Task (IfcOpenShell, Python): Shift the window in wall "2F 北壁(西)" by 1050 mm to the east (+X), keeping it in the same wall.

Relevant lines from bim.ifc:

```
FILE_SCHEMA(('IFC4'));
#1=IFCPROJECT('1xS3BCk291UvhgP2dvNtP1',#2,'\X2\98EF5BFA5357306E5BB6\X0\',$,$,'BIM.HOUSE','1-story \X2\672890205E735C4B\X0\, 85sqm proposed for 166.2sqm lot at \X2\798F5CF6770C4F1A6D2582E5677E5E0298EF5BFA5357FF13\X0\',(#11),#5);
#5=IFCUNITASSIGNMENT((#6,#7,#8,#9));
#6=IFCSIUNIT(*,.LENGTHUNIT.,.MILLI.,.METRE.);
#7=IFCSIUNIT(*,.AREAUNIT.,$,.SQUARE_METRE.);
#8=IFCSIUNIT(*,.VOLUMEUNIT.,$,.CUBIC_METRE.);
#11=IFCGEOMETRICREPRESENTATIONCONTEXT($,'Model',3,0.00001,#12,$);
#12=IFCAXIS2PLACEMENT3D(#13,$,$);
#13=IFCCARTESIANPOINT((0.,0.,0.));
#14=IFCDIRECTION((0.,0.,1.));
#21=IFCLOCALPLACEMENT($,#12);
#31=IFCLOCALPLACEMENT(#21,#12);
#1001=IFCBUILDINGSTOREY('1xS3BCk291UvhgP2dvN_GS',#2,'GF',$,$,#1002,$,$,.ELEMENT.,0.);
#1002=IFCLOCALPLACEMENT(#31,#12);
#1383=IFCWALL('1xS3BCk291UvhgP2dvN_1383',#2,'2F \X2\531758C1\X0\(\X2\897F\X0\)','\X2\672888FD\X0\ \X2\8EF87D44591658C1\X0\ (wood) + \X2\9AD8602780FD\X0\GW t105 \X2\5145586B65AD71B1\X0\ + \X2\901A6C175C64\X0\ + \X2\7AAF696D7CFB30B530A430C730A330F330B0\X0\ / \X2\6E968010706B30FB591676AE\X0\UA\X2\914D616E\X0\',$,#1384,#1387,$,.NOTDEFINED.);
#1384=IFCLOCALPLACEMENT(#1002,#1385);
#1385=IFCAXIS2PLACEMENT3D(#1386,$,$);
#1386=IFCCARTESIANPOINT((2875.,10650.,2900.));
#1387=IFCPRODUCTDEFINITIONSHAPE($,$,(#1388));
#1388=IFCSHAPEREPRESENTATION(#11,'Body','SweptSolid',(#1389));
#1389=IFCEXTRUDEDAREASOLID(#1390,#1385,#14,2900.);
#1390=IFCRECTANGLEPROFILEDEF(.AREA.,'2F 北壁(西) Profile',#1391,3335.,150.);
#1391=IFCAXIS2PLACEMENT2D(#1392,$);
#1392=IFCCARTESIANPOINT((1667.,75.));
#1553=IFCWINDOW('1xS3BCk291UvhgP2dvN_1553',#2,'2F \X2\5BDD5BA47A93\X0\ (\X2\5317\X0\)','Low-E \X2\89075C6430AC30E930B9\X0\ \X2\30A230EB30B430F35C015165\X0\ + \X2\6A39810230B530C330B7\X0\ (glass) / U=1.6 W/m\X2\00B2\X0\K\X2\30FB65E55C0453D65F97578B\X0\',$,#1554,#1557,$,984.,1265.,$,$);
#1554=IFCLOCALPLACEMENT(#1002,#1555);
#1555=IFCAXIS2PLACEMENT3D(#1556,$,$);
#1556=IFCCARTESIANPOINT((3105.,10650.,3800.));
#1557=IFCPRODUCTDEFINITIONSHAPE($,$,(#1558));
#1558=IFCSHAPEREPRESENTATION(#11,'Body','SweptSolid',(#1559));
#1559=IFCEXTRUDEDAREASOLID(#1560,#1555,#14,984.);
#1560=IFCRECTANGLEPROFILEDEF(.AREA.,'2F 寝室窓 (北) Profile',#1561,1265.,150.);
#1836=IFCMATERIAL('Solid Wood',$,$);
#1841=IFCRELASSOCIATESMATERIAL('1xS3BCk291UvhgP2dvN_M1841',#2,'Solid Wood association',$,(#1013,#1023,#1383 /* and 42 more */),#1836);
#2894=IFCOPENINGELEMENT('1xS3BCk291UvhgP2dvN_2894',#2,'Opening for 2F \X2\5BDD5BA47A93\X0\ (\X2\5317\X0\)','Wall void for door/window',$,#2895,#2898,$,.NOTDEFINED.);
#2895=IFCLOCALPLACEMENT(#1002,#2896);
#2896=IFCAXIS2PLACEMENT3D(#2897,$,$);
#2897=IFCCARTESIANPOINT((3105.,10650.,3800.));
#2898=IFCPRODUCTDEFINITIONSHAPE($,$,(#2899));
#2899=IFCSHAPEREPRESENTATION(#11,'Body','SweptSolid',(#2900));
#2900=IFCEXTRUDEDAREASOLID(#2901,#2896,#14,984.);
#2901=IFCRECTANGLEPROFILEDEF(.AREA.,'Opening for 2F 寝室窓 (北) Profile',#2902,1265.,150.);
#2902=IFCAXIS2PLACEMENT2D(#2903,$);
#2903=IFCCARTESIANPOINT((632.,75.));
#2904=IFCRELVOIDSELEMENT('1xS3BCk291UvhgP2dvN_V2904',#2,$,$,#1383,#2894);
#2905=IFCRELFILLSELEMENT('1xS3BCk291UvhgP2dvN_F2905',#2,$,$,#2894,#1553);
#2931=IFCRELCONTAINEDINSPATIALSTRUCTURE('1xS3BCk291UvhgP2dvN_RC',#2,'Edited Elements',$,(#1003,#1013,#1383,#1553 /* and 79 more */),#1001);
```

```python
import ifcopenshell
import ifcopenshell.api.geometry
import ifcopenshell.util.placement
import ifcopenshell.util.unit

model = ifcopenshell.open("bim.ifc")
unit_scale = ifcopenshell.util.unit.calculate_unit_scale(model)

window = model.by_id(1553)
opening = window.FillsVoids[0].RelatingOpeningElement
wall = opening.VoidsElements[0].RelatingBuildingElement

wall_matrix = ifcopenshell.util.placement.get_local_placement(wall.ObjectPlacement)
shift = wall_matrix[:3, 0] * 1.05 / unit_scale
before = ifcopenshell.util.placement.get_local_placement(window.ObjectPlacement)[:3, 3].copy()

# The window is not placed relative to its opening, so move both.
for product in (opening, window):
    matrix = ifcopenshell.util.placement.get_local_placement(product.ObjectPlacement)
    matrix[:3, 3] += shift
    ifcopenshell.api.geometry.edit_object_placement(model, product=product, matrix=matrix, is_si=False)

after = ifcopenshell.util.placement.get_local_placement(window.ObjectPlacement)[:3, 3]
print("window moved by", (after - before).round(3) + 0.0)

model.write("bim-out.ifc")
```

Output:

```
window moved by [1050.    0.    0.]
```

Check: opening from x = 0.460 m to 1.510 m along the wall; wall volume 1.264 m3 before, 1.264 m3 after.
